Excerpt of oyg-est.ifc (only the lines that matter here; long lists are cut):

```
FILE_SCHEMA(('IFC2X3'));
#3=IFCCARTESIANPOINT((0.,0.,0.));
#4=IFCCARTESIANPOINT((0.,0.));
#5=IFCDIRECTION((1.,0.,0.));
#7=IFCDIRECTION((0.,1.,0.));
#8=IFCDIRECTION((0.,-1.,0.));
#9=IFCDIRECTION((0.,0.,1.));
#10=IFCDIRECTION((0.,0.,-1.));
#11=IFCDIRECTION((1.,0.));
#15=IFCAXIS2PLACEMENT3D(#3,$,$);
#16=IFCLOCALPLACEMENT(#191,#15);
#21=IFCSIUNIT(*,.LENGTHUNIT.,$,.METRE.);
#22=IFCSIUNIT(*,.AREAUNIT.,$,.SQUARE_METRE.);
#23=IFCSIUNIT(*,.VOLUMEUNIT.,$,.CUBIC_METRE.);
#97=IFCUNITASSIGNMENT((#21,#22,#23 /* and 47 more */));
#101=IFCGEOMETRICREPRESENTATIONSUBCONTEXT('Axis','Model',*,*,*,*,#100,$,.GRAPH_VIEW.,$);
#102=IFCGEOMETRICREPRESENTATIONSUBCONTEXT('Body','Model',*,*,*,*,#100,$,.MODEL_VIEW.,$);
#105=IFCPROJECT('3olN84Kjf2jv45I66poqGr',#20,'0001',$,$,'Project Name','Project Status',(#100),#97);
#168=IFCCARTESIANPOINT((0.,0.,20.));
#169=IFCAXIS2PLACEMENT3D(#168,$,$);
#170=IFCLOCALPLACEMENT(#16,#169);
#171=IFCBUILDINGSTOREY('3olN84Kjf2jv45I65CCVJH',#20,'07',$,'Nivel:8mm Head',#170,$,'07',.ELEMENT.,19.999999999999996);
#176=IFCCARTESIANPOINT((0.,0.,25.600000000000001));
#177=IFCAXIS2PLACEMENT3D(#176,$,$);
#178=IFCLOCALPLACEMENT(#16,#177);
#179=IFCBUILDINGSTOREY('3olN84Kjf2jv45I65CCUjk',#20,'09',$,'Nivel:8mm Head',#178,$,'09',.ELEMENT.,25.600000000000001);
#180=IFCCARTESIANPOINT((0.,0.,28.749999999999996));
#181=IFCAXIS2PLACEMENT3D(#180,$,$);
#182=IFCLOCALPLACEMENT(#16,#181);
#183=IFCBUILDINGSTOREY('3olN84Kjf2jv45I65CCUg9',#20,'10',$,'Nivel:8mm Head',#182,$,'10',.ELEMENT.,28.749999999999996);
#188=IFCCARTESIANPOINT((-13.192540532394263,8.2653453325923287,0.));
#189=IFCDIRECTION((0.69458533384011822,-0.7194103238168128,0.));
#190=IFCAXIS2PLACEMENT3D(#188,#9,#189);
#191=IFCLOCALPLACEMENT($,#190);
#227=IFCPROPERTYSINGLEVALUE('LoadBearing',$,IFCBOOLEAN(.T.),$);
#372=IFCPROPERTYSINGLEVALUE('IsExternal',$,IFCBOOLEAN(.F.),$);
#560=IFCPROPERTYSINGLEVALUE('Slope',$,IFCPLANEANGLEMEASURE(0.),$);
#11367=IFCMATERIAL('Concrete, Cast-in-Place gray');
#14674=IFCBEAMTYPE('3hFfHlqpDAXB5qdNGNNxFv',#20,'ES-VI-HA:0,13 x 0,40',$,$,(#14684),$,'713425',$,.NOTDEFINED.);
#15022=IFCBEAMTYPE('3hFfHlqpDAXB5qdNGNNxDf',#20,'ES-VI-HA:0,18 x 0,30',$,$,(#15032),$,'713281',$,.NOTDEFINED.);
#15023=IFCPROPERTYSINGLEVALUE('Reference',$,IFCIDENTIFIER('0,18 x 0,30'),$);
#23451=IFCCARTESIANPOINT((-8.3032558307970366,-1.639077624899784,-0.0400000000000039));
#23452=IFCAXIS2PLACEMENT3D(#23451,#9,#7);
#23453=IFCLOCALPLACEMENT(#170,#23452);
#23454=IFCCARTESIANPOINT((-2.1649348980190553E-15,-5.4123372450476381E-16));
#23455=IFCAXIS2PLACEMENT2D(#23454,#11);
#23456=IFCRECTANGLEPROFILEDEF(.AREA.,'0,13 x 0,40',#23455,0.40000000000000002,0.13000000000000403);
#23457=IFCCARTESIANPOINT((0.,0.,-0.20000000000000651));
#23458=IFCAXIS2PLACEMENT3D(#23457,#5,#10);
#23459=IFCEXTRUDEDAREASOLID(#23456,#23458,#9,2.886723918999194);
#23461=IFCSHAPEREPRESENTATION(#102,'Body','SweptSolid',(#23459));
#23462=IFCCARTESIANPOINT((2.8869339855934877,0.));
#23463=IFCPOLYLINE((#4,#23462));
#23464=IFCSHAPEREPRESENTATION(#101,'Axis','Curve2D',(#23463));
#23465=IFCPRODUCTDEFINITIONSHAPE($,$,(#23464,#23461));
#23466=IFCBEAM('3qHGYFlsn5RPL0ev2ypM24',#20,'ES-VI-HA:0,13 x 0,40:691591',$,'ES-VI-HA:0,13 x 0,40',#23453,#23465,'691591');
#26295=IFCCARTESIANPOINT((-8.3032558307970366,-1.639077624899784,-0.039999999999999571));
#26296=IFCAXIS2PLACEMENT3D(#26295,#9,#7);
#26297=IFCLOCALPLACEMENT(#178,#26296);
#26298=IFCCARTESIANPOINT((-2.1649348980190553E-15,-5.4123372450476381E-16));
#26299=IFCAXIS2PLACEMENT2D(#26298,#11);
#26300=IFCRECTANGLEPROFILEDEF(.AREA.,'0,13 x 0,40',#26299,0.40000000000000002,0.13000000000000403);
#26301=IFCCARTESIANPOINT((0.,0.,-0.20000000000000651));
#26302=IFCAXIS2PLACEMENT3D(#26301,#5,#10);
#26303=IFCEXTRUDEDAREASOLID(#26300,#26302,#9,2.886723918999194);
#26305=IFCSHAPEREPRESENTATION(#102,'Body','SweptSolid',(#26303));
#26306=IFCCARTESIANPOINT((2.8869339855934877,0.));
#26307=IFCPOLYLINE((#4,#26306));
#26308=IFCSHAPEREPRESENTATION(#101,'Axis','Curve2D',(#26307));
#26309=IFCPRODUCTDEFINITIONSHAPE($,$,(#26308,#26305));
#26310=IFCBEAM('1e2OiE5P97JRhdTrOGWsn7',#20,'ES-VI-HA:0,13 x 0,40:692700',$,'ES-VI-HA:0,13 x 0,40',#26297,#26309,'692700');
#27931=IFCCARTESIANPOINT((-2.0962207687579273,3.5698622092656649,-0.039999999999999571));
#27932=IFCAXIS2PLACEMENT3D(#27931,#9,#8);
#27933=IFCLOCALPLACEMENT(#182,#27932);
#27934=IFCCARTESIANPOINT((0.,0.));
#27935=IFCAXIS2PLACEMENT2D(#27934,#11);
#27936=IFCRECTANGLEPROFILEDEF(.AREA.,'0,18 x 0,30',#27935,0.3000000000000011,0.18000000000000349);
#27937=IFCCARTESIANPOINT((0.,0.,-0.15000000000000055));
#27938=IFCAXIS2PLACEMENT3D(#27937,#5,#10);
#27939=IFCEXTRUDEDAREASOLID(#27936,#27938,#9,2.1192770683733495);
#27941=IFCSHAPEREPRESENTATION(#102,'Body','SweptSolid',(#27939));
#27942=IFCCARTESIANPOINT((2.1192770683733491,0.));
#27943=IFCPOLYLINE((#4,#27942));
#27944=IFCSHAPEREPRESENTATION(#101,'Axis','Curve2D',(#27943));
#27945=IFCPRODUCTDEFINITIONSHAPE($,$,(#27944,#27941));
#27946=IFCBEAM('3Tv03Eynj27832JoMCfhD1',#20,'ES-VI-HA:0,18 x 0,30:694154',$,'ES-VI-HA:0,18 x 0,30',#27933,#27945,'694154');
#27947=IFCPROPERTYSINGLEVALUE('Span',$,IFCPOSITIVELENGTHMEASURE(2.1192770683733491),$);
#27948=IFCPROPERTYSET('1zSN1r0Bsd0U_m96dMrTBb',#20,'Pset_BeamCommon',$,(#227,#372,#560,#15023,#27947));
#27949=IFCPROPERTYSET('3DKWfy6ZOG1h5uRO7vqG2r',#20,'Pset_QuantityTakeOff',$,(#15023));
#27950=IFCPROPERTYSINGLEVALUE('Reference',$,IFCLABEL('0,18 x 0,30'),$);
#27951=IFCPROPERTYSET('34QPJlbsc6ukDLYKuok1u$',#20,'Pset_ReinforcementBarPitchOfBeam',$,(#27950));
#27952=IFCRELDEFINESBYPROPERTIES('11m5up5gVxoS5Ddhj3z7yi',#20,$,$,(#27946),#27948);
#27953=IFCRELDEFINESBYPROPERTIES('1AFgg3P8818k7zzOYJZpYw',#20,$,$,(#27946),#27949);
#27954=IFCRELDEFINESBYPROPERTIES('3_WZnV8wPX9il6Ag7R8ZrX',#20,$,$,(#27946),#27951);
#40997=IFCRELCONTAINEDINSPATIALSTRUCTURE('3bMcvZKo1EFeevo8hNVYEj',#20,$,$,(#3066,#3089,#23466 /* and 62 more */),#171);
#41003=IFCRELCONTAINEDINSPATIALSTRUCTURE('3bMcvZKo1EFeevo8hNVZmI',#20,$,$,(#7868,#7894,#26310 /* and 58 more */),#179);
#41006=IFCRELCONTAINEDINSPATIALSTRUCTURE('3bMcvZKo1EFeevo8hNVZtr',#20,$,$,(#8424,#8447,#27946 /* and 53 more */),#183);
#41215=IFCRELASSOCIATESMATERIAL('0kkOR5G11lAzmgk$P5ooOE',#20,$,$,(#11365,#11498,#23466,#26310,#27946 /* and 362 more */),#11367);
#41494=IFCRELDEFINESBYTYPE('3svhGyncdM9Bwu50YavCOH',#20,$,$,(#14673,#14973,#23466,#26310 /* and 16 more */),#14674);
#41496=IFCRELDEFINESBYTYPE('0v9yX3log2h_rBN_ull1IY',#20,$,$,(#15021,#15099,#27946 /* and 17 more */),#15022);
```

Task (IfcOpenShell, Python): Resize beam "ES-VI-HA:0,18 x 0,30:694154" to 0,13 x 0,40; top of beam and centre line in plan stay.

```python
import ifcopenshell
import ifcopenshell.api.pset
import ifcopenshell.api.type
import ifcopenshell.util.element
import ifcopenshell.util.representation

model = ifcopenshell.open("oyg-est.ifc")

member = model.by_guid("3Tv03Eynj27832JoMCfhD1")
source = next(p for p in model.by_type("IfcRectangleProfileDef") if p.ProfileName == "0,13 x 0,40")

body = ifcopenshell.util.representation.get_representation(member, "Model", "Body")
solid = body.Items[0]
old_profile = solid.SweptArea

# Copy the section's sizes but keep this member's own profile position.
profile = ifcopenshell.util.element.copy(model, source)
# Profiles are centred, so shift by half the change in depth to hold the top.
shift = (old_profile.XDim - profile.XDim) / 2
x, y = old_profile.Position.Location.Coordinates
up = (-1.0, 0.0)  # upwards, in the solid's own plane
location = model.createIfcCartesianPoint((x + up[0] * shift, y + up[1] * shift))
profile.Position = model.createIfcAxis2Placement2D(location, old_profile.Position.RefDirection)
solid.SweptArea = profile
if not model.get_total_inverses(old_profile):
    ifcopenshell.util.element.remove_deep2(model, old_profile)

new_type = model.by_guid("3hFfHlqpDAXB5qdNGNNxFv")
ifcopenshell.api.type.assign_type(
    model, related_objects=[member], relating_type=new_type, should_map_representations=False
)
member.Name = member.Name.replace("0,18 x 0,30", "0,13 x 0,40")
member.ObjectType = "ES-VI-HA:0,13 x 0,40"
pset = model.by_id(ifcopenshell.util.element.get_pset(member, "Pset_BeamCommon", should_inherit=False)["id"])
ifcopenshell.api.pset.edit_pset(model, pset=pset, properties={"Reference": "0,13 x 0,40"})
pset = model.by_id(ifcopenshell.util.element.get_pset(member, "Pset_QuantityTakeOff", should_inherit=False)["id"])
ifcopenshell.api.pset.edit_pset(model, pset=pset, properties={"Reference": "0,13 x 0,40"})
pset = model.by_id(ifcopenshell.util.element.get_pset(member, "Pset_ReinforcementBarPitchOfBeam", should_inherit=False)["id"])
ifcopenshell.api.pset.edit_pset(model, pset=pset, properties={"Reference": "0,13 x 0,40"})

print(solid.SweptArea)

model.write("oyg-est_v2.ifc")
```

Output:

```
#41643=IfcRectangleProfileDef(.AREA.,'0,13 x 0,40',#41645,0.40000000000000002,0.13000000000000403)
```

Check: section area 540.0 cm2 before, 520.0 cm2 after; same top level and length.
